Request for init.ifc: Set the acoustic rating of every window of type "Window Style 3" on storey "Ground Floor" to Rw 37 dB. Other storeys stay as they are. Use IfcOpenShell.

First a look at what the model holds.

```python
import ifcopenshell
import ifcopenshell.util.element

model = ifcopenshell.open("init.ifc")
print(model.schema)
storey = next(s for s in model.by_type("IfcBuildingStorey") if s.Name == "Ground Floor")
windows = [e for e in ifcopenshell.util.element.get_decomposition(storey) if e.is_a("IfcWindow")]
seen = {}
for e in windows:
    element_type = ifcopenshell.util.element.get_type(e)
    key = (element_type.Name if element_type != e and element_type else None, ifcopenshell.util.element.get_pset(e, "Pset_WindowCommon", "AcousticRating"))
    seen[key] = seen.get(key, 0) + 1
for (name, value), count in sorted(seen.items(), key=str):
    print(count, "x", name, "|", value)
```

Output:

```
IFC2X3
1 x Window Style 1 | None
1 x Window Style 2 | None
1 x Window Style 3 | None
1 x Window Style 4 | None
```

```python
import ifcopenshell
import ifcopenshell.api.pset
import ifcopenshell.util.element

model = ifcopenshell.open("init.ifc")

storey = next(s for s in model.by_type("IfcBuildingStorey") if s.Name == "Ground Floor")
windows = [e for e in ifcopenshell.util.element.get_decomposition(storey) if e.is_a("IfcWindow")]

count = 0
for e in windows:
    element_type = ifcopenshell.util.element.get_type(e)
    if element_type in (None, e) or element_type.Name != "Window Style 3":
        continue
    # add_pset returns the element's existing set when there is one.
    pset = ifcopenshell.api.pset.add_pset(model, product=e, name="Pset_WindowCommon")
    ifcopenshell.api.pset.edit_pset(model, pset=pset, properties={"AcousticRating": "Rw 37 dB"})
    count += 1

print(count, "windows updated")

model.write("init-out.ifc")
```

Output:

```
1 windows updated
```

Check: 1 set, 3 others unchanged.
